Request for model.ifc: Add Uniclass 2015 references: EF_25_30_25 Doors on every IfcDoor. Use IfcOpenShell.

First a look at what the model holds.

```python
import ifcopenshell

model = ifcopenshell.open("model.ifc")
print(model.schema)
print("classifications:", [c.Name for c in model.by_type("IfcClassification")])
for ifc_class in ("IfcDoor", "IfcRoof", "IfcStair", "IfcWall", "IfcWindow"):
    print(ifc_class, len(model.by_type(ifc_class)))
```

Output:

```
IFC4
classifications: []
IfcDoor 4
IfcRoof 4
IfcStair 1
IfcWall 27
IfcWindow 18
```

```python
import ifcopenshell
import ifcopenshell.api.classification

model = ifcopenshell.open("model.ifc")

system = ifcopenshell.api.classification.add_classification(model, classification="Uniclass 2015")

codes = {
    "IfcDoor": ("EF_25_30_25", "Doors"),
}
for ifc_class, (code, name) in codes.items():
    products = model.by_type(ifc_class)
    ifcopenshell.api.classification.add_reference(
        model, products=products, classification=system, identification=code, name=name
    )
    print(code, len(products))

model.write("model_v2.ifc")
```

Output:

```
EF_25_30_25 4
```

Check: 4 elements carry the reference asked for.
